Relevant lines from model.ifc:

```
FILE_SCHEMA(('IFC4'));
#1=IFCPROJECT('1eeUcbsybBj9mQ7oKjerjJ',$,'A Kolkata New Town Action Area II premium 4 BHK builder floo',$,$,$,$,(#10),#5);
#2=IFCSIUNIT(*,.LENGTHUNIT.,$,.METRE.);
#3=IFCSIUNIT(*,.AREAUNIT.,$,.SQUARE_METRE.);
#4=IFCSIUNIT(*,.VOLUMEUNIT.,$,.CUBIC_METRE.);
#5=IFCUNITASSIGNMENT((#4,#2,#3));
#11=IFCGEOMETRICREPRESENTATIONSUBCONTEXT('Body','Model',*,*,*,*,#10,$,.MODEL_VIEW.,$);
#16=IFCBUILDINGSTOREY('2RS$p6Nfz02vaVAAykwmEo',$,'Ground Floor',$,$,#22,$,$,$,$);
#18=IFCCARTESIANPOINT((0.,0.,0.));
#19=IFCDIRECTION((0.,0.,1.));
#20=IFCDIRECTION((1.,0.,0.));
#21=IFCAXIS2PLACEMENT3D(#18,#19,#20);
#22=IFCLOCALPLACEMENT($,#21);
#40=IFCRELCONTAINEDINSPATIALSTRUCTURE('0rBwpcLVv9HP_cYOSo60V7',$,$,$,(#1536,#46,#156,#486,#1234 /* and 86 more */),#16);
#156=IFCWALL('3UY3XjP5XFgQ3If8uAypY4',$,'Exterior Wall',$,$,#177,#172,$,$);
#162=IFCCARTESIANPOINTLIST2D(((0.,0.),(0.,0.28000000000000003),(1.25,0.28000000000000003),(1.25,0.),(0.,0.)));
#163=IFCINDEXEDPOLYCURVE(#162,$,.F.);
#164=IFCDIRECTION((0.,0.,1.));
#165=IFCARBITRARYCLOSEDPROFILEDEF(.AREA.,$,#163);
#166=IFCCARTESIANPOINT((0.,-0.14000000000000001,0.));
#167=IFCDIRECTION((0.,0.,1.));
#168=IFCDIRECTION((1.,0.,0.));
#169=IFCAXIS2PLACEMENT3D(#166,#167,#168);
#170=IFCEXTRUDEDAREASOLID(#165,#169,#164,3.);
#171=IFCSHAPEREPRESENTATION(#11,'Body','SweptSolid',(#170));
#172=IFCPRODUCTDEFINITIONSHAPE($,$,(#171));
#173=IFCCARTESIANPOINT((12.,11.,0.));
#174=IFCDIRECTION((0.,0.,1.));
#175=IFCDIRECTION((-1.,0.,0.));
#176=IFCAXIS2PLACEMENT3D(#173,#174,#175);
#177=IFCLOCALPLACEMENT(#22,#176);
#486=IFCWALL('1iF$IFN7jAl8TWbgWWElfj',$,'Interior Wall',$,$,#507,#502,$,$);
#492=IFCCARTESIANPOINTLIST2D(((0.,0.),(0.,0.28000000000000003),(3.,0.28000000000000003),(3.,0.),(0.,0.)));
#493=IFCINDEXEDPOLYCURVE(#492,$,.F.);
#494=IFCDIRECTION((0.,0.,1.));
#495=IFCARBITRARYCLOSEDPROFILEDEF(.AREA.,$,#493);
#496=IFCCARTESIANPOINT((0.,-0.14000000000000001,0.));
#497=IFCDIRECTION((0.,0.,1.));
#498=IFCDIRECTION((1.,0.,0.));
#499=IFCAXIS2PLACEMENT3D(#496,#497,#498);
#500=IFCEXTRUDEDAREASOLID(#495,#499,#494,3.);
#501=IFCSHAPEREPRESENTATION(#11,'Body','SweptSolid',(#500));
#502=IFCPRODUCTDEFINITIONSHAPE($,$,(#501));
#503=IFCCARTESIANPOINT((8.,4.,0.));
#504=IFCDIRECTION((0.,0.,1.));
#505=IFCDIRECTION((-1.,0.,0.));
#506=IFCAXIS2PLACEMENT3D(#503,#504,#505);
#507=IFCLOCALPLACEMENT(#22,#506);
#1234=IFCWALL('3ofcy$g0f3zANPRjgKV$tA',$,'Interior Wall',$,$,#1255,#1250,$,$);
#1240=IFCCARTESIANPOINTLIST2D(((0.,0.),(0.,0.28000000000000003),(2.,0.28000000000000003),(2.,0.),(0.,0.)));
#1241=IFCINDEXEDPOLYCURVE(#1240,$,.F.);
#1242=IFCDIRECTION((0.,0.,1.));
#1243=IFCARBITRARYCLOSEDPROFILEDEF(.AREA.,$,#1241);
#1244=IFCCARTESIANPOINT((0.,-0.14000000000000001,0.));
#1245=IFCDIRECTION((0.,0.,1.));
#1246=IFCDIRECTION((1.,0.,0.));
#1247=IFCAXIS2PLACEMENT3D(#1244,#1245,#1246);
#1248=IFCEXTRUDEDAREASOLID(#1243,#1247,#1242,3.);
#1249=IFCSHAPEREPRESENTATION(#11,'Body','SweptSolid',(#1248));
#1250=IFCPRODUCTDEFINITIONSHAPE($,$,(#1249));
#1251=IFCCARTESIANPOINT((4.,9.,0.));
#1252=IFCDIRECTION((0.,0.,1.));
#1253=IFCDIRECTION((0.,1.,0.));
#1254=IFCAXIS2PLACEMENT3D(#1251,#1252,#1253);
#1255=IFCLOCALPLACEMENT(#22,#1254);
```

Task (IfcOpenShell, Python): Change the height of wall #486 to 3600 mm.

```python
import ifcopenshell
import ifcopenshell.geom
import ifcopenshell.util.representation
import ifcopenshell.util.shape

model = ifcopenshell.open("model.ifc")
settings = ifcopenshell.geom.settings()


def volume(element):
    """Net volume in cubic metres, openings subtracted."""
    shape = ifcopenshell.geom.create_shape(settings, element)
    return ifcopenshell.util.shape.get_volume(shape.geometry)


wall = model.by_id(486)
before = volume(wall)

body = ifcopenshell.util.representation.get_representation(wall, "Model", "Body")
solid = body.Items[0]
old_height = solid.Depth
solid.Depth = 3.6
after = volume(wall)

print(f"height {old_height:g} -> {solid.Depth:g}, volume {before:.3f} -> {after:.3f} m3")

model.write("model_rev.ifc")
```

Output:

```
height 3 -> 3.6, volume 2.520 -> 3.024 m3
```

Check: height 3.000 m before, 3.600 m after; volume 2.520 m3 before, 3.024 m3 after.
